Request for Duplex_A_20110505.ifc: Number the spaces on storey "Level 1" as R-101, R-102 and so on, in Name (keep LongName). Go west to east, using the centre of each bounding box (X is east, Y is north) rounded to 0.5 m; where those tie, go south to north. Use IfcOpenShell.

First a look at what the model holds.

```python
import ifcopenshell
import ifcopenshell.util.element
import ifcopenshell.util.placement

model = ifcopenshell.open("Duplex_A_20110505.ifc")
print(model.schema)
storey = next(s for s in model.by_type("IfcBuildingStorey") if s.Name == "Level 1")
spaces = [e for e in ifcopenshell.util.element.get_decomposition(storey) if e.is_a("IfcSpace")]
for e in sorted(spaces, key=lambda e: e.id()):
    origin = ifcopenshell.util.placement.get_local_placement(e.ObjectPlacement)[:3, 3]
    print(e.id(), e.Name, e.LongName, origin.round(2) + 0.0, sep=" | ")
```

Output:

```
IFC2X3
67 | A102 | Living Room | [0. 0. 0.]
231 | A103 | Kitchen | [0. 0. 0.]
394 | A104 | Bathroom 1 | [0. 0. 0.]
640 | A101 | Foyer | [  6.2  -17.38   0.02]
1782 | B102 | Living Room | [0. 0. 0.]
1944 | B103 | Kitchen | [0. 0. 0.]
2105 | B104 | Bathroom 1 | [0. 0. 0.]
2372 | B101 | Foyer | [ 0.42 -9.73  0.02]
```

```python
import ifcopenshell
import ifcopenshell.geom
import ifcopenshell.util.element
import ifcopenshell.util.shape

model = ifcopenshell.open("Duplex_A_20110505.ifc")
settings = ifcopenshell.geom.settings()
settings.set("use-world-coords", True)


def centre(element):
    shape = ifcopenshell.geom.create_shape(settings, element)
    return ifcopenshell.util.shape.get_bbox_centroid(shape.geometry)


storey = next(s for s in model.by_type("IfcBuildingStorey") if s.Name == "Level 1")
spaces = [e for e in ifcopenshell.util.element.get_decomposition(storey) if e.is_a("IfcSpace")]

# Insertion points can sit at a corner or the storey origin, so sort by the geometry (in metres).
centres = {e: centre(e) for e in spaces}
spaces.sort(key=lambda e: (round(centres[e][0] / 0.5), centres[e][1]))

for i, e in enumerate(spaces, start=1):
    number = f"R-1{i:02d}"
    e.Name = number
    print(e.id(), number)

model.write("Duplex_A_20110505_edited.ifc")
```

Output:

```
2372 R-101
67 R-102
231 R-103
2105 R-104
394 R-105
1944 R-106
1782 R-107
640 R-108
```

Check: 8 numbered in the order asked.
